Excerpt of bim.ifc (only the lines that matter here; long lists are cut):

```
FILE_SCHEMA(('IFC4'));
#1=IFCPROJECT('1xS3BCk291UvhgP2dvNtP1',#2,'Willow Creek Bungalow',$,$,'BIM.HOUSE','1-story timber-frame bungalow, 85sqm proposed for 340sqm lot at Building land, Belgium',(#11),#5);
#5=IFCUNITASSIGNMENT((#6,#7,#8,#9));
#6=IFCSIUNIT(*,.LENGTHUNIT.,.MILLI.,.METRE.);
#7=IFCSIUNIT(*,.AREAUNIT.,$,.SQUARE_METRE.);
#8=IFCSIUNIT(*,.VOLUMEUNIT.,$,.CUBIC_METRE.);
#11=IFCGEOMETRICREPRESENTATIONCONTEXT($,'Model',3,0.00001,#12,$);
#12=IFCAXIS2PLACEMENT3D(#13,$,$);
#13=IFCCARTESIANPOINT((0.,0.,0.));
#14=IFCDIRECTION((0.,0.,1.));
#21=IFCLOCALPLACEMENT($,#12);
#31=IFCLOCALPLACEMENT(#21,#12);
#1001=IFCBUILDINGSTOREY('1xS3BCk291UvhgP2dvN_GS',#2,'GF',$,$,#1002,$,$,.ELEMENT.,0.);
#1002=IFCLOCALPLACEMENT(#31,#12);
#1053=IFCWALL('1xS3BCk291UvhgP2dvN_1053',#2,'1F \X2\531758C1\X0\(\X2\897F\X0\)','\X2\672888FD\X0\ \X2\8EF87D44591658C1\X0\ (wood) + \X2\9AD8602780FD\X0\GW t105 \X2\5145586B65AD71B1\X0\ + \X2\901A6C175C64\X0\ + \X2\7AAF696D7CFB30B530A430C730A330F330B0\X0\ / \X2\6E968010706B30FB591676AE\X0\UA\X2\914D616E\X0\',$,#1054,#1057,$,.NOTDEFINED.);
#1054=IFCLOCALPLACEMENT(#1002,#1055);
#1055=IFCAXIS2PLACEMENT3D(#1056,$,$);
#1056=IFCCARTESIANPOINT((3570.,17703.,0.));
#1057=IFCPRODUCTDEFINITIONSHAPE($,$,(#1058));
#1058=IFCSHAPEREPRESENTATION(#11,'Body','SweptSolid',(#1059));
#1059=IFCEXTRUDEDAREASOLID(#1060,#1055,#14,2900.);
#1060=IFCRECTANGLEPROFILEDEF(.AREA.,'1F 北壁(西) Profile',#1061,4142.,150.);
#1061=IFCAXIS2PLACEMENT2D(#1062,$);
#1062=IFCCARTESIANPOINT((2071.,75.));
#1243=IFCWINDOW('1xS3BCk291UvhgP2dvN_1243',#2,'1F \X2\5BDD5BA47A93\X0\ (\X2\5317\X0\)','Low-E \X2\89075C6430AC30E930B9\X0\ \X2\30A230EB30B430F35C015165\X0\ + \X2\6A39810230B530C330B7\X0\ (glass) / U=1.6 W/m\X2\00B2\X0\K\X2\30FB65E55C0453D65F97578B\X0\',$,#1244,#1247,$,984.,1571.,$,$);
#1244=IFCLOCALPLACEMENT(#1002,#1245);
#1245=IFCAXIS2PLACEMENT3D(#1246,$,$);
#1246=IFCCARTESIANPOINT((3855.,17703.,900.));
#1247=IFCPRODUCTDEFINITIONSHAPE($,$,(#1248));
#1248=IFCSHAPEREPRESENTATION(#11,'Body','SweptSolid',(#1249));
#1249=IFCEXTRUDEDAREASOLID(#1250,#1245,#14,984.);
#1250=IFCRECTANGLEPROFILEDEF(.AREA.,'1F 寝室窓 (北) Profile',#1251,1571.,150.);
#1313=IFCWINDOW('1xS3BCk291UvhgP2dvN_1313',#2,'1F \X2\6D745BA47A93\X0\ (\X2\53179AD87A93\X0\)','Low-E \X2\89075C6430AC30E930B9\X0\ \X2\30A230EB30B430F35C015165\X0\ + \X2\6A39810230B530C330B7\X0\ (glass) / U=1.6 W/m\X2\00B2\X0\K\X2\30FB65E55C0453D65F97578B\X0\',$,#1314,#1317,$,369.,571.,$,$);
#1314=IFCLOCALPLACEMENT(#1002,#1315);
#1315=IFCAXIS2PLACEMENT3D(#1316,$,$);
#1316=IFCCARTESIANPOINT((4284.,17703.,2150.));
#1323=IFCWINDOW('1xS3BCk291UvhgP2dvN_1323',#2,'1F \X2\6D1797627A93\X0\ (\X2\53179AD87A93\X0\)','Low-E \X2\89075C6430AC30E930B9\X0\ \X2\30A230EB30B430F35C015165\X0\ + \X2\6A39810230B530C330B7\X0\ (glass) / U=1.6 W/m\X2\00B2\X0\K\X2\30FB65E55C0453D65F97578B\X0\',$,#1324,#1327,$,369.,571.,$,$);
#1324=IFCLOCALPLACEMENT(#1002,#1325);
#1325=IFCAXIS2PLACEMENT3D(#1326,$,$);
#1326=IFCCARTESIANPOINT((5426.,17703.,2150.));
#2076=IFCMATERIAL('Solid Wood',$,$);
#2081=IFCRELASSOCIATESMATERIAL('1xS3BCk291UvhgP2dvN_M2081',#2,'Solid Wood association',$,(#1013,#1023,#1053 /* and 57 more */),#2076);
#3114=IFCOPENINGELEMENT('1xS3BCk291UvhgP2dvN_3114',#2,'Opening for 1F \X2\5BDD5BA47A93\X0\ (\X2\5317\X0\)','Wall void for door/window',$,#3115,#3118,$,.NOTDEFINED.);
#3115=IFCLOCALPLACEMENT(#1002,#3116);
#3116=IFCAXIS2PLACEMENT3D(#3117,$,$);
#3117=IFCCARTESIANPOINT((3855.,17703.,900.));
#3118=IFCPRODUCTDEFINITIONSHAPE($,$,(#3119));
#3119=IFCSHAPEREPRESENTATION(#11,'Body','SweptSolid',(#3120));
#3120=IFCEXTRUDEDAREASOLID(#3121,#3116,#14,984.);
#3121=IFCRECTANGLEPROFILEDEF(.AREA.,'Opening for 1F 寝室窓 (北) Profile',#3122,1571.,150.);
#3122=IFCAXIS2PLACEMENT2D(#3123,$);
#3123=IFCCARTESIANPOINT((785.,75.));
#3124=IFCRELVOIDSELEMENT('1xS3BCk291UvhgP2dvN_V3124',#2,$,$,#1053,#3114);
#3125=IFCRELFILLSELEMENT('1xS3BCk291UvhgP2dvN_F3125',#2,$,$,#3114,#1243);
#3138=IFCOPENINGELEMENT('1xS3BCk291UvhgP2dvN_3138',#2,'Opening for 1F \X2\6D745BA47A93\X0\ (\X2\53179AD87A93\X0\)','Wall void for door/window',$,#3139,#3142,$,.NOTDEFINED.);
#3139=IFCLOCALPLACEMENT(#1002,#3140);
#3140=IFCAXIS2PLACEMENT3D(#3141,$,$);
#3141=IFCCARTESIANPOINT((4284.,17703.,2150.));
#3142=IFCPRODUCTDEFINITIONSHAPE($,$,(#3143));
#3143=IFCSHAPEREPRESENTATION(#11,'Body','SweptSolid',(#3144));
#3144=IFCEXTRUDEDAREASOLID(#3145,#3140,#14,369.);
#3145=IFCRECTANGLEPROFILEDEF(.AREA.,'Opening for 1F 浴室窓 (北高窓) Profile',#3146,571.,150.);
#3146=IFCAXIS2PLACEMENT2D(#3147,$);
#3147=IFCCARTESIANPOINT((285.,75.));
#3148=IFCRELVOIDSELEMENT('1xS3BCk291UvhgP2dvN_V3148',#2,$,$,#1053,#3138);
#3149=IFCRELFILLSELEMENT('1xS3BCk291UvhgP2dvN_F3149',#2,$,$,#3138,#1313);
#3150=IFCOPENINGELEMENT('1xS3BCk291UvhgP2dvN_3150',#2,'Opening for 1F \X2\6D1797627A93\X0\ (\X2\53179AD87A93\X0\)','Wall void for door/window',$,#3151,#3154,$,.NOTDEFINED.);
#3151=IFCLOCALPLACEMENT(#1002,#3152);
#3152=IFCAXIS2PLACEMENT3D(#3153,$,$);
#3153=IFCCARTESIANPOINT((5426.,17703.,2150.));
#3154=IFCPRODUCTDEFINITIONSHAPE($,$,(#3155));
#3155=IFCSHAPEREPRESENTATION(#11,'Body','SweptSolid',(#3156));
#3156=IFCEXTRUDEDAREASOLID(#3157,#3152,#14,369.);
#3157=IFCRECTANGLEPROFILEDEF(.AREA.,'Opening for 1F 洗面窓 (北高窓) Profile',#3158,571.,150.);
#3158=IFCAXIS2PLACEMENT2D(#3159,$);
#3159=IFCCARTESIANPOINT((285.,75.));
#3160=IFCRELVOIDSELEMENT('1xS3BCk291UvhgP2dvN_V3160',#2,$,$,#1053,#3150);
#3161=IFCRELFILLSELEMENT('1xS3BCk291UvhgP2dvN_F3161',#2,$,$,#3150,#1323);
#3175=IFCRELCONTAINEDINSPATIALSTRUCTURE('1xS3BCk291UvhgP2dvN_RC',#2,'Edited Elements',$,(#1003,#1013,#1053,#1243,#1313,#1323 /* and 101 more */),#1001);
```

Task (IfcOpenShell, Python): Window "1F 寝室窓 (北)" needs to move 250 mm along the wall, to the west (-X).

```python
import ifcopenshell
import ifcopenshell.api.geometry
import ifcopenshell.util.placement
import ifcopenshell.util.unit

model = ifcopenshell.open("bim.ifc")
unit_scale = ifcopenshell.util.unit.calculate_unit_scale(model)

window = model.by_guid("1xS3BCk291UvhgP2dvN_1243")
opening = window.FillsVoids[0].RelatingOpeningElement
wall = opening.VoidsElements[0].RelatingBuildingElement

wall_matrix = ifcopenshell.util.placement.get_local_placement(wall.ObjectPlacement)
shift = wall_matrix[:3, 0] * -0.25 / unit_scale
before = ifcopenshell.util.placement.get_local_placement(window.ObjectPlacement)[:3, 3].copy()

# The window is not placed relative to its opening, so move both.
for product in (opening, window):
    matrix = ifcopenshell.util.placement.get_local_placement(product.ObjectPlacement)
    matrix[:3, 3] += shift
    ifcopenshell.api.geometry.edit_object_placement(model, product=product, matrix=matrix, is_si=False)

after = ifcopenshell.util.placement.get_local_placement(window.ObjectPlacement)[:3, 3]
print("window moved by", (after - before).round(3) + 0.0)

model.write("bim_edited.ifc")
```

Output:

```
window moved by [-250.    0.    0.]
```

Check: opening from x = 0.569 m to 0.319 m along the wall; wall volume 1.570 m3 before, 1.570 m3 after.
